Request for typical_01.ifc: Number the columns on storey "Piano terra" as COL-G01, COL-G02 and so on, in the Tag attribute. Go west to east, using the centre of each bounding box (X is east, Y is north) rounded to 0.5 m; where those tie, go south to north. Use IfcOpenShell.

First a look at what the model holds.

```python
import ifcopenshell
import ifcopenshell.util.element
import ifcopenshell.util.placement

model = ifcopenshell.open("typical_01.ifc")
print(model.schema)
storey = next(s for s in model.by_type("IfcBuildingStorey") if s.Name == "Piano terra")
columns = [e for e in ifcopenshell.util.element.get_decomposition(storey) if e.is_a("IfcColumn")]
for e in sorted(columns, key=lambda e: e.id()):
    origin = ifcopenshell.util.placement.get_local_placement(e.ObjectPlacement)[:3, 3]
    print(e.id(), e.Tag, e.Name, origin.round(2) + 0.0, sep=" | ")
```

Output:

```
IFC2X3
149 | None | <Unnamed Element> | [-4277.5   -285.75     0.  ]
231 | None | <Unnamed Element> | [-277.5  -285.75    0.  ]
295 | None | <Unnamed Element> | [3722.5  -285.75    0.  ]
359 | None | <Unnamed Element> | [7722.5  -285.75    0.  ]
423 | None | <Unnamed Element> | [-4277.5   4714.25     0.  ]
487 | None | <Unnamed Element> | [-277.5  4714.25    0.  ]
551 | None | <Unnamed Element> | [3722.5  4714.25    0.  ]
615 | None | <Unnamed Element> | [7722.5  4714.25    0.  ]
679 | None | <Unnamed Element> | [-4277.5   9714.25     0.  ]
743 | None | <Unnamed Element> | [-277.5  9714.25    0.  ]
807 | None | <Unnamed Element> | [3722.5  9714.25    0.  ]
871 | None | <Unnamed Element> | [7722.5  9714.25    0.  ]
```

```python
import ifcopenshell
import ifcopenshell.geom
import ifcopenshell.util.element
import ifcopenshell.util.shape

model = ifcopenshell.open("typical_01.ifc")
settings = ifcopenshell.geom.settings()
settings.set("use-world-coords", True)


def centre(element):
    shape = ifcopenshell.geom.create_shape(settings, element)
    return ifcopenshell.util.shape.get_bbox_centroid(shape.geometry)


storey = next(s for s in model.by_type("IfcBuildingStorey") if s.Name == "Piano terra")
columns = [e for e in ifcopenshell.util.element.get_decomposition(storey) if e.is_a("IfcColumn")]

# Insertion points can sit at a corner or the storey origin, so sort by the geometry (in metres).
centres = {e: centre(e) for e in columns}
columns.sort(key=lambda e: (round(centres[e][0] / 0.5), centres[e][1]))

for i, e in enumerate(columns, start=1):
    number = f"COL-G{i:02d}"
    e.Tag = number
    print(e.id(), number)

model.write("typical_01_v2.ifc")
```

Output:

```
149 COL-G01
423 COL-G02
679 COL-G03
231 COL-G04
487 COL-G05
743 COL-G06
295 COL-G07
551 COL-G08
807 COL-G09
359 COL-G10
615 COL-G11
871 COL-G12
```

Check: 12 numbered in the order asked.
